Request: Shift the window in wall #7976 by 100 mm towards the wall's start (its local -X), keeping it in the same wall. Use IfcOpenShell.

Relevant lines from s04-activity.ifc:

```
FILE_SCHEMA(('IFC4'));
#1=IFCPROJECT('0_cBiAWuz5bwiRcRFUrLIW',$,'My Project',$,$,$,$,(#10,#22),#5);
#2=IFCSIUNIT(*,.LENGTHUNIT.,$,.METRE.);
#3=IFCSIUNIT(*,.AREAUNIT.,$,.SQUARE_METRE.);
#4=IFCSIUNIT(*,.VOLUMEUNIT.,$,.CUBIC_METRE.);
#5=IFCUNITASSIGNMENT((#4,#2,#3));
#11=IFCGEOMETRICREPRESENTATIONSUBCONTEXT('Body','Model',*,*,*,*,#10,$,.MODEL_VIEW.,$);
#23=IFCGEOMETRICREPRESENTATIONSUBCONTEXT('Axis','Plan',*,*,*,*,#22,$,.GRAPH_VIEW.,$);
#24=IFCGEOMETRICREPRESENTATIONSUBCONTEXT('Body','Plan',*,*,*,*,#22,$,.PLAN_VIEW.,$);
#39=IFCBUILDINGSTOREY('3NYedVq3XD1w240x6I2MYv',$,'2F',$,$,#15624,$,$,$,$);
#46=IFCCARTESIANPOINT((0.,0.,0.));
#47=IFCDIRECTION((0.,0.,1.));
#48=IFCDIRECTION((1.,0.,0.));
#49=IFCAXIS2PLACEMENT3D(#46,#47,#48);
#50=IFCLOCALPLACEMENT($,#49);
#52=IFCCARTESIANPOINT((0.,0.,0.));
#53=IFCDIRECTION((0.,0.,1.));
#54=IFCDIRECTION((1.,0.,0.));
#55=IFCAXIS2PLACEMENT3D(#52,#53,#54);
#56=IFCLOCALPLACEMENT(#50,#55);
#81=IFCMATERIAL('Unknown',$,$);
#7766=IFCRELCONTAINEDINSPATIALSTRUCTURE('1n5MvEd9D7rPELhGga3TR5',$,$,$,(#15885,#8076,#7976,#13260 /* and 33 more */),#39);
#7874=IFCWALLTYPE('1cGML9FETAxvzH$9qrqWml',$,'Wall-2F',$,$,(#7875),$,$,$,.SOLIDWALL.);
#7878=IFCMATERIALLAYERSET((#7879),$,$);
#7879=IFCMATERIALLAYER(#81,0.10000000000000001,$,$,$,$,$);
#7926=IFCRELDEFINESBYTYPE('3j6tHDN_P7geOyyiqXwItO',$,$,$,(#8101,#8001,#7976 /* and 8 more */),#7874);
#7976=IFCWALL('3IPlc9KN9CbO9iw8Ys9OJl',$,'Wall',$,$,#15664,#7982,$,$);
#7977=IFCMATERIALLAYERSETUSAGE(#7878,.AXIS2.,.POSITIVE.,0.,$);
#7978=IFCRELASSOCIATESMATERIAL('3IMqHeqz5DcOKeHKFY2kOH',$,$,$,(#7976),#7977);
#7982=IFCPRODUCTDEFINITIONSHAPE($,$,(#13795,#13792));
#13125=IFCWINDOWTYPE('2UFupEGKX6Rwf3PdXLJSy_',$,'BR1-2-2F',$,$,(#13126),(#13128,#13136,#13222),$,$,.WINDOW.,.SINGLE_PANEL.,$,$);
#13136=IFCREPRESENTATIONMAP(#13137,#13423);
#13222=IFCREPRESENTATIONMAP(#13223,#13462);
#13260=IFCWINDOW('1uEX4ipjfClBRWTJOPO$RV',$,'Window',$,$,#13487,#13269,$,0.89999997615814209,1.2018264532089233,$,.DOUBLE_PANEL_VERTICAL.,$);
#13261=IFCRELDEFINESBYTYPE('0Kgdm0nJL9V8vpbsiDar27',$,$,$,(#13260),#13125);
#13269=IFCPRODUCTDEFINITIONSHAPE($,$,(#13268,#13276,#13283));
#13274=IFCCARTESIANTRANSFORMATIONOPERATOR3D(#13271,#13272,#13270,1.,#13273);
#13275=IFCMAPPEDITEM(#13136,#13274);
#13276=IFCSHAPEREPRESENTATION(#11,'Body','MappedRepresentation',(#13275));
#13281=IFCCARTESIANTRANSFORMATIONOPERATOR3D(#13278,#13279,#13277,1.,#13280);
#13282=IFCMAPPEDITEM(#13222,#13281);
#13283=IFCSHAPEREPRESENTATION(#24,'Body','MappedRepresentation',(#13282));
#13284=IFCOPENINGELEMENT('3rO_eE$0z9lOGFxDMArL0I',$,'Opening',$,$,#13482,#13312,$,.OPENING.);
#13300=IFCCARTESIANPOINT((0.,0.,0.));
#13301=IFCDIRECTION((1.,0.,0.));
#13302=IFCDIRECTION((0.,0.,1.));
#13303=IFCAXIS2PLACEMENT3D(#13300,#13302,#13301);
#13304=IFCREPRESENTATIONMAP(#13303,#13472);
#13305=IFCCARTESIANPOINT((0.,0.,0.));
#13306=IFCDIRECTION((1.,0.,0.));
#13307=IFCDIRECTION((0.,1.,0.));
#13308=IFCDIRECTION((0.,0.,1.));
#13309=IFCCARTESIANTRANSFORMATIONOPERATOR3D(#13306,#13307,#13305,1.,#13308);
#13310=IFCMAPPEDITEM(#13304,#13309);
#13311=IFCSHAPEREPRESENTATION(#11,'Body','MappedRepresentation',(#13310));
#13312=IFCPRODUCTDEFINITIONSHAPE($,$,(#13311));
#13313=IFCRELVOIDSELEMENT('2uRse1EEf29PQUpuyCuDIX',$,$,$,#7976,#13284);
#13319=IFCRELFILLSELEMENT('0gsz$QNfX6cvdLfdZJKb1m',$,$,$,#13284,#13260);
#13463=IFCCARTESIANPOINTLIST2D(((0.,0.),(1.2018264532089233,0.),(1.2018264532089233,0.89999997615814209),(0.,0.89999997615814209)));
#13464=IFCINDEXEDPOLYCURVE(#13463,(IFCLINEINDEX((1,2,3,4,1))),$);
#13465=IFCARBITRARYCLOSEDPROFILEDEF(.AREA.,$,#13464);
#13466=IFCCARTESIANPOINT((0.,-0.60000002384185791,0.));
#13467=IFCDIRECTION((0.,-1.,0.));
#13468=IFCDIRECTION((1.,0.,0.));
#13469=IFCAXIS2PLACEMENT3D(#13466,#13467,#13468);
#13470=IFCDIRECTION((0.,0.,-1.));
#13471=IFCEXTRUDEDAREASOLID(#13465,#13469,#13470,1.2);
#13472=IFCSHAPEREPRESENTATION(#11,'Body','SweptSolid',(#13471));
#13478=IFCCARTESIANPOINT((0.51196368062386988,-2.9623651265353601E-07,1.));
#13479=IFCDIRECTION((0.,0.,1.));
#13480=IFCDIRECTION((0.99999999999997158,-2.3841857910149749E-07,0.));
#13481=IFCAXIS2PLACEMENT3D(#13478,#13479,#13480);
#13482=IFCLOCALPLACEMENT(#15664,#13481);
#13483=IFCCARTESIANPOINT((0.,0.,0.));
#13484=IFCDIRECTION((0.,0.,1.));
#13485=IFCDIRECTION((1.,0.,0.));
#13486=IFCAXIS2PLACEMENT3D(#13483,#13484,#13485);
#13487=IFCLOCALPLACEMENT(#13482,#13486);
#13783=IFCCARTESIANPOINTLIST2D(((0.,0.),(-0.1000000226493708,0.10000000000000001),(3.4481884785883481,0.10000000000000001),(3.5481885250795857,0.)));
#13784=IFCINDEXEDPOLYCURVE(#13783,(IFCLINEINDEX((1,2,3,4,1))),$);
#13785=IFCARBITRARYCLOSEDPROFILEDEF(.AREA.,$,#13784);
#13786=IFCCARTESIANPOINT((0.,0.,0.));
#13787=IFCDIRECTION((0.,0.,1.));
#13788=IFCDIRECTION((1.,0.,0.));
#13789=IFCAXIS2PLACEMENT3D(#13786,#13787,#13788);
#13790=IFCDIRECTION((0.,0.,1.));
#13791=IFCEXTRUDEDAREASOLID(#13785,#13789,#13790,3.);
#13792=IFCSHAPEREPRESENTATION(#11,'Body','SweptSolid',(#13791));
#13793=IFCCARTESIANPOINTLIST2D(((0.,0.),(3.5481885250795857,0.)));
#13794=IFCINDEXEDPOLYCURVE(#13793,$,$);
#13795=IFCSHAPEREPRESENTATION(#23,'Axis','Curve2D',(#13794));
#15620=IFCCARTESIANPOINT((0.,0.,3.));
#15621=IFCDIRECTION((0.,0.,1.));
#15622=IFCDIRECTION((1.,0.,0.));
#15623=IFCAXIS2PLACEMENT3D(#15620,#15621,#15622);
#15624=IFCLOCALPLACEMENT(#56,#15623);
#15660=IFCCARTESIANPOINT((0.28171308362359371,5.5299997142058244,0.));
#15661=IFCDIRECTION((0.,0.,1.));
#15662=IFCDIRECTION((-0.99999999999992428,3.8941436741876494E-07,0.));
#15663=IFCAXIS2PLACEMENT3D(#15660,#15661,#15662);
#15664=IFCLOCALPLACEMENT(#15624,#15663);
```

```python
import ifcopenshell
import ifcopenshell.api.geometry
import ifcopenshell.util.placement

model = ifcopenshell.open("s04-activity.ifc")

window = model.by_guid("1uEX4ipjfClBRWTJOPO$RV")
opening = window.FillsVoids[0].RelatingOpeningElement
wall = opening.VoidsElements[0].RelatingBuildingElement

wall_matrix = ifcopenshell.util.placement.get_local_placement(wall.ObjectPlacement)
shift = wall_matrix[:3, 0] * -0.1
before = ifcopenshell.util.placement.get_local_placement(window.ObjectPlacement)[:3, 3].copy()

# The window is placed relative to its opening, so it follows when the opening moves.
matrix = ifcopenshell.util.placement.get_local_placement(opening.ObjectPlacement)
matrix[:3, 3] += shift
ifcopenshell.api.geometry.edit_object_placement(
    model, product=opening, matrix=matrix, is_si=False, should_transform_children=True
)

after = ifcopenshell.util.placement.get_local_placement(window.ObjectPlacement)[:3, 3]
print("window moved by", (after - before).round(3) + 0.0)

model.write("s04-activity_updated.ifc")
```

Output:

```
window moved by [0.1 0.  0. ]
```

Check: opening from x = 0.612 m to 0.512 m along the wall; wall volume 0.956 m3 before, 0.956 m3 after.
